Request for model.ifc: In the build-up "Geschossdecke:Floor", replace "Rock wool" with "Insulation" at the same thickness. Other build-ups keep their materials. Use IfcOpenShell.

First a look at what the model holds.

```python
import ifcopenshell
import ifcopenshell.util.element

model = ifcopenshell.open("model.ifc")
print(model.schema)
for layer_set in model.by_type("IfcMaterialLayerSet"):
    if layer_set.LayerSetName == "Geschossdecke:Floor":
        for layer in layer_set.MaterialLayers:
            print(layer.id(), layer.Material and layer.Material.Name, layer.LayerThickness, sep=" | ")
        print(len(ifcopenshell.util.element.get_elements_by_material(model, layer_set)), "elements and types use it")
print(sorted(m.Name for m in model.by_type("IfcMaterial") if m.Name)[:60])
```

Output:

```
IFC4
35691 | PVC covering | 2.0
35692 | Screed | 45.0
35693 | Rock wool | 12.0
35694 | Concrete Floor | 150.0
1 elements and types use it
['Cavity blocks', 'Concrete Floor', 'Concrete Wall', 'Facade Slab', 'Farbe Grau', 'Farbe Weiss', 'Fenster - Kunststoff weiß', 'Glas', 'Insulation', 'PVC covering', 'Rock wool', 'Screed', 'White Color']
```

```python
import ifcopenshell
import ifcopenshell.api.material

model = ifcopenshell.open("model.ifc")

layer_set = next(s for s in model.by_type("IfcMaterialLayerSet") if s.LayerSetName == "Geschossdecke:Floor")
layer = next(l for l in layer_set.MaterialLayers if l.Material and l.Material.Name == "Rock wool")
material = next(m for m in model.by_type("IfcMaterial") if m.Name == "Insulation")

# Point this one layer at the other material; renaming the old one would change it everywhere.
ifcopenshell.api.material.edit_layer(model, layer=layer, attributes={}, material=material)

print([l.Material.Name if l.Material else None for l in layer_set.MaterialLayers])

model.write("model_edited.ifc")
```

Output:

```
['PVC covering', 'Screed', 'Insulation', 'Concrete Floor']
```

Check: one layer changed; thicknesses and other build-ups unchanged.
